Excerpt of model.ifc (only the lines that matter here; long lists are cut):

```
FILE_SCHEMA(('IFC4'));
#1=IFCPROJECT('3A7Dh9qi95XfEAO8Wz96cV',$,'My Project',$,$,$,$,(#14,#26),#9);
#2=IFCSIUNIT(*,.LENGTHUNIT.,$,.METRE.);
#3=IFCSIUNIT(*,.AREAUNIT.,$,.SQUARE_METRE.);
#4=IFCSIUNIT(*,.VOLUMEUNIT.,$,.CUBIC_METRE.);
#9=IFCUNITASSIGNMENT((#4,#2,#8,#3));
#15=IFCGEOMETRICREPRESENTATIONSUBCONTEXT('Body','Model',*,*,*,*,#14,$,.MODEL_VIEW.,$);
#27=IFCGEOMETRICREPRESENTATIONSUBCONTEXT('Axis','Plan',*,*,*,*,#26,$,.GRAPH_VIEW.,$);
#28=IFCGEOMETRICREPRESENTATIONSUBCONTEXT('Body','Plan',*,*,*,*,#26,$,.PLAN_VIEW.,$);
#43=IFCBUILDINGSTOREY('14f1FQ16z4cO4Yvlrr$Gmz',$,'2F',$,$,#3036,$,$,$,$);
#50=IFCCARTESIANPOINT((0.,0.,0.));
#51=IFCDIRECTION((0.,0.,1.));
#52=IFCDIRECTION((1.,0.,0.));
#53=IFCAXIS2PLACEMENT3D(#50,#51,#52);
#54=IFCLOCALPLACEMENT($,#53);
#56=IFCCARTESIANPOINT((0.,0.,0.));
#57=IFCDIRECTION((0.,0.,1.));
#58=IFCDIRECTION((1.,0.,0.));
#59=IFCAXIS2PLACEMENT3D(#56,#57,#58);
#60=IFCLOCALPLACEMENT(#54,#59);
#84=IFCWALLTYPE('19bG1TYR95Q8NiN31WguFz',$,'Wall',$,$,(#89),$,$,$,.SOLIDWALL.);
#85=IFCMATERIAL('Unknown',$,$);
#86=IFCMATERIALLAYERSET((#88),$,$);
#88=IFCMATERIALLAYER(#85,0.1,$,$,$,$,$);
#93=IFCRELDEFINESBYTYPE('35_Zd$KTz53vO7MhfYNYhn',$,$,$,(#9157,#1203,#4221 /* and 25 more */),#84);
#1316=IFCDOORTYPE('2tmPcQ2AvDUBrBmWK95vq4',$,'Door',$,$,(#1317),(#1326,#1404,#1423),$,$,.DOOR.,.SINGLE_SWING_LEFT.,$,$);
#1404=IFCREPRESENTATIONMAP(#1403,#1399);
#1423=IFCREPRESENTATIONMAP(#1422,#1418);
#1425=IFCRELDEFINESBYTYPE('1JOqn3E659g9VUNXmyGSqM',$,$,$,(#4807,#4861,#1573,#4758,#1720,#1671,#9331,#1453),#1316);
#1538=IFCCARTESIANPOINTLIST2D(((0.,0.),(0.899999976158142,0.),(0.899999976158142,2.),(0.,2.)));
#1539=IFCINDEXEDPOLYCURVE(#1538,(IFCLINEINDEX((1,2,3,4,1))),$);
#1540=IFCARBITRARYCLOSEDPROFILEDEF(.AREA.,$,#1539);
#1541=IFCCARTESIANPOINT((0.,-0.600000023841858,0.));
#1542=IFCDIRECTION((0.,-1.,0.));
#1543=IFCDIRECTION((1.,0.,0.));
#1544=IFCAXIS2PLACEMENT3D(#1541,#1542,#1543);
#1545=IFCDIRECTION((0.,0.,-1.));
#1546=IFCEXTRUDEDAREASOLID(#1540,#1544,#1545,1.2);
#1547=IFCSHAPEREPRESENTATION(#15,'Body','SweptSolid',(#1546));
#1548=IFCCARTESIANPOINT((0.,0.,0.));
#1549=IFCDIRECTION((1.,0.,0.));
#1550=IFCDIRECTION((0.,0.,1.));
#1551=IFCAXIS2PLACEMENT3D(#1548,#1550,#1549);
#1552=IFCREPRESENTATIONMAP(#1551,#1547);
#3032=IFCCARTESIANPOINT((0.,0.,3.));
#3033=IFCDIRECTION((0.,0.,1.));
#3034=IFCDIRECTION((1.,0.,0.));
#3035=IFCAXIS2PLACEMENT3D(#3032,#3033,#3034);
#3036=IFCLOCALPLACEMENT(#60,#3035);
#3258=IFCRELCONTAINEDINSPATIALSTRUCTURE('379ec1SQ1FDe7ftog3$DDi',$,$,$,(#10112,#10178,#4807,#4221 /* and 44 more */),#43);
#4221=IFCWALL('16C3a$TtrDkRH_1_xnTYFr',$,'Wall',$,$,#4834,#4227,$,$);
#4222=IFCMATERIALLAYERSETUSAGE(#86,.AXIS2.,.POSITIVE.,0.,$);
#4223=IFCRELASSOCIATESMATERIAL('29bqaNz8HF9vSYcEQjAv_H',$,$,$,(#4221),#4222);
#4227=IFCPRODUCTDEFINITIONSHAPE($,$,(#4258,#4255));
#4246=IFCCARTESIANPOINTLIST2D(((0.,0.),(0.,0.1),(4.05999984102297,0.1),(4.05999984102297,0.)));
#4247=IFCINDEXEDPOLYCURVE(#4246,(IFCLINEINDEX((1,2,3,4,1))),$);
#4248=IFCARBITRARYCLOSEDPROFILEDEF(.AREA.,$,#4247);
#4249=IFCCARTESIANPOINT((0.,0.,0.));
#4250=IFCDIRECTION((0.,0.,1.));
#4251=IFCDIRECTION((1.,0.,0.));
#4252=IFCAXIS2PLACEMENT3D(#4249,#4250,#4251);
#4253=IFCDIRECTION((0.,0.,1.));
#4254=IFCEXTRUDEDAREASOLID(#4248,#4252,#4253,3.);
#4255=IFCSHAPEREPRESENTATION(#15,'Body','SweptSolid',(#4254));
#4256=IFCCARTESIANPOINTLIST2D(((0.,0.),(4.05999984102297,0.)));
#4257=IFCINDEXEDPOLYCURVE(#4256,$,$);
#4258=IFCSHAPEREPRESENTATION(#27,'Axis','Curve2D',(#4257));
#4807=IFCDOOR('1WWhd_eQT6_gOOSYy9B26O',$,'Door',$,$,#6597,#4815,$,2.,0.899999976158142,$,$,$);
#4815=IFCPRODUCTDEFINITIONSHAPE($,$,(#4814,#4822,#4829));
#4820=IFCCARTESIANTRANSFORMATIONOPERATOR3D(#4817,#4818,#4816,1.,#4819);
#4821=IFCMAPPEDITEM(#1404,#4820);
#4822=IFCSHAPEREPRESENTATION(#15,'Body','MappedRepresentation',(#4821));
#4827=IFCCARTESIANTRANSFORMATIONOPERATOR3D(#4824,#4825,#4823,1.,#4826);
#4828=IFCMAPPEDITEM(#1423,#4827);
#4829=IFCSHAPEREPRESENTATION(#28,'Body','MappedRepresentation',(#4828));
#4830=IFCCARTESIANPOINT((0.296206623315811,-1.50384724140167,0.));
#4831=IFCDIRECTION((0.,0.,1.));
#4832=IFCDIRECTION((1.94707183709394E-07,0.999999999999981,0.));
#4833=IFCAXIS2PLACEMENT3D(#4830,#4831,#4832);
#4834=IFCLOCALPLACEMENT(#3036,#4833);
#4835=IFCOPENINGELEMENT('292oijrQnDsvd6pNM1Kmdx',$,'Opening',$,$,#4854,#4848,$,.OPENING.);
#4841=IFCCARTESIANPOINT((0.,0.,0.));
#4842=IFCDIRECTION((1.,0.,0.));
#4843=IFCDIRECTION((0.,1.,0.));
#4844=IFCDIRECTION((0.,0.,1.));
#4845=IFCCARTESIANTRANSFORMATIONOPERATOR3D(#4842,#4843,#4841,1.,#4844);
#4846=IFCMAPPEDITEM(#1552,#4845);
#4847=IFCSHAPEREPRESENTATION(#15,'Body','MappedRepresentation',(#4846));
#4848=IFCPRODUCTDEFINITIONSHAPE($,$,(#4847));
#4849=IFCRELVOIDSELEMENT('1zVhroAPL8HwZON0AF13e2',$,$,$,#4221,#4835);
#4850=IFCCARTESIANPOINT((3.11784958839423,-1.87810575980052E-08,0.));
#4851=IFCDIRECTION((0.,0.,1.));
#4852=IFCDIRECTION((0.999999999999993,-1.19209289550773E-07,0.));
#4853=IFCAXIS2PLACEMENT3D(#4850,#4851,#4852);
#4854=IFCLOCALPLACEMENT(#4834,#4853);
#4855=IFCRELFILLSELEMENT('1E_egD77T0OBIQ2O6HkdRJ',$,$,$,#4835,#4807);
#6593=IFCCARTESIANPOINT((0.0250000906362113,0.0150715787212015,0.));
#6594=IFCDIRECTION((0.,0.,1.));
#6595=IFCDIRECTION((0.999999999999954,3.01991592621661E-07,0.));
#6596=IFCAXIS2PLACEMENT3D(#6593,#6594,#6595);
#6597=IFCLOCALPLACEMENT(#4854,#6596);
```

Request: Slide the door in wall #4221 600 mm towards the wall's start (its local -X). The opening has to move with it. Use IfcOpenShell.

```python
import ifcopenshell
import ifcopenshell.api.geometry
import ifcopenshell.util.placement
import ifcopenshell.util.unit

model = ifcopenshell.open("model.ifc")
unit_scale = ifcopenshell.util.unit.calculate_unit_scale(model)

door = model.by_id(4807)
opening = door.FillsVoids[0].RelatingOpeningElement
wall = opening.VoidsElements[0].RelatingBuildingElement

wall_matrix = ifcopenshell.util.placement.get_local_placement(wall.ObjectPlacement)
shift = wall_matrix[:3, 0] * -0.6 / unit_scale
before = ifcopenshell.util.placement.get_local_placement(door.ObjectPlacement)[:3, 3].copy()

# The door is placed relative to its opening, so it follows when the opening moves.
matrix = ifcopenshell.util.placement.get_local_placement(opening.ObjectPlacement)
matrix[:3, 3] += shift
ifcopenshell.api.geometry.edit_object_placement(
    model, product=opening, matrix=matrix, is_si=False, should_transform_children=True
)

after = ifcopenshell.util.placement.get_local_placement(door.ObjectPlacement)[:3, 3]
print("door moved by", (after - before).round(3) + 0.0)

model.write("model_rev.ifc")
```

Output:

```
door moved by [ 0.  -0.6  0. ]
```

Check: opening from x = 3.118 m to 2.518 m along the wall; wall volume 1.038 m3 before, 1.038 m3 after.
